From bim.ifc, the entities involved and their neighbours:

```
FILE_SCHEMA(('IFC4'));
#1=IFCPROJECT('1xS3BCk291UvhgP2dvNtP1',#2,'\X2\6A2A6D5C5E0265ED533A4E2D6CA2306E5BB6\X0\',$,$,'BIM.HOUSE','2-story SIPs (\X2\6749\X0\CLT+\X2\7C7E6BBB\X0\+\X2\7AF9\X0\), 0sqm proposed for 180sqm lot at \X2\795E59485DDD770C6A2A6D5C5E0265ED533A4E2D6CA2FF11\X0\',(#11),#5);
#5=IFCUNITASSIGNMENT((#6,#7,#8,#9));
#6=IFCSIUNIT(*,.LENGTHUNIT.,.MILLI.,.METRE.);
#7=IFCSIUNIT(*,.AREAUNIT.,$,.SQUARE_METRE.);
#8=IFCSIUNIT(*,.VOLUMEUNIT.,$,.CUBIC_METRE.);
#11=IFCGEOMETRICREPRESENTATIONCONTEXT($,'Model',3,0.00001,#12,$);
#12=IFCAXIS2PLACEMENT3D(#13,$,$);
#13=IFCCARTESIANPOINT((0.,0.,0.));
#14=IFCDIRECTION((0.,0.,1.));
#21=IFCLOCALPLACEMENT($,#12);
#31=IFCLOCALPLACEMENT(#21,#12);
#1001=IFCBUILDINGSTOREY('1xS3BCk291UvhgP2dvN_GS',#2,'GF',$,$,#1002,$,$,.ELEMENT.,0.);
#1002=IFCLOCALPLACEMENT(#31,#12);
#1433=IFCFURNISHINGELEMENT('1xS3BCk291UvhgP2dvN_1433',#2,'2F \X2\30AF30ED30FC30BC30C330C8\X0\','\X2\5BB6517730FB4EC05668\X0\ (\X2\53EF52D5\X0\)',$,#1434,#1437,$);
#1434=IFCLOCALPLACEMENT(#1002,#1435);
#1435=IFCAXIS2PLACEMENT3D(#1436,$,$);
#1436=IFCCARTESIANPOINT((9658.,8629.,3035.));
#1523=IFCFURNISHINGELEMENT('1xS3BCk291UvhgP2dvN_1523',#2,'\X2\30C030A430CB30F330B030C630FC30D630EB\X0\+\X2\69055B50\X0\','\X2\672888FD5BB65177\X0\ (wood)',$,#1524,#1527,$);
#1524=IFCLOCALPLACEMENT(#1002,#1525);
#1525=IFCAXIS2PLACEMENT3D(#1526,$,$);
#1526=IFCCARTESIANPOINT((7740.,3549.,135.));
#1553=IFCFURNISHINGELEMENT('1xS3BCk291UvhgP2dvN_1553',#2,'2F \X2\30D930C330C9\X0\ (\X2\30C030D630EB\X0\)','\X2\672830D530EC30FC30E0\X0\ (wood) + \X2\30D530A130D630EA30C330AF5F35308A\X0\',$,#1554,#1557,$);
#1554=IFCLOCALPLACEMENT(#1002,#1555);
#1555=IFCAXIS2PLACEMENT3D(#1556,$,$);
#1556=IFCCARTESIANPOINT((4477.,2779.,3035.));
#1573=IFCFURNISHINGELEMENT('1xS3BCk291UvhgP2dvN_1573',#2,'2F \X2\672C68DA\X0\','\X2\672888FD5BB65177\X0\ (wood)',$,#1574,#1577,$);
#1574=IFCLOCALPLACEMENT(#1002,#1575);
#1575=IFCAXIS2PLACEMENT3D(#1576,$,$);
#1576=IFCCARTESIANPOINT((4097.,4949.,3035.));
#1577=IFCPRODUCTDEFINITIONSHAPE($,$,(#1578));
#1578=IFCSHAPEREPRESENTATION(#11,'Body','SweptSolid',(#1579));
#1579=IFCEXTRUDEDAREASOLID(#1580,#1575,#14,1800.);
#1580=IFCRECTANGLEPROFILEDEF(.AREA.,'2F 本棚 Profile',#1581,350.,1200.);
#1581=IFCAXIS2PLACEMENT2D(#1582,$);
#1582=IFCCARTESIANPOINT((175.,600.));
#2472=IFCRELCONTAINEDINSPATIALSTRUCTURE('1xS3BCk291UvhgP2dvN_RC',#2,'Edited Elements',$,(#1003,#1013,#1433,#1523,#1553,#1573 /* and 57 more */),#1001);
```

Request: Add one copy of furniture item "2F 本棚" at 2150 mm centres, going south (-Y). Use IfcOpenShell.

```python
import numpy as np
import ifcopenshell
import ifcopenshell.api.geometry
import ifcopenshell.api.root
import ifcopenshell.util.element
import ifcopenshell.util.placement
import ifcopenshell.util.unit

model = ifcopenshell.open("bim.ifc")
unit_scale = ifcopenshell.util.unit.calculate_unit_scale(model)


def reuse_history(source, copy):
    """copy_class also copies each property set's owner history, people and application; keep the originals."""
    for rel in copy.IsDefinedBy:
        if rel.is_a("IfcRelDefinesByProperties") and (history := rel.RelatingPropertyDefinition.OwnerHistory):
            rel.RelatingPropertyDefinition.OwnerHistory = source.OwnerHistory
            ifcopenshell.util.element.remove_deep2(model, history)


source = model.by_guid("1xS3BCk291UvhgP2dvN_1573")
base = ifcopenshell.util.placement.get_local_placement(source.ObjectPlacement)
step = np.array([0.0, -1.0, 0.0]) * 2.15 / unit_scale

for i in range(1, 2):
    copy = ifcopenshell.api.root.copy_class(model, product=source)
    copy.Representation = ifcopenshell.util.element.copy_deep(
        model, source.Representation, exclude=["IfcGeometricRepresentationContext", "IfcRepresentationMap"]
    )
    reuse_history(source, copy)
    matrix = base.copy()
    matrix[:3, 3] += i * step
    print("added at", matrix[:3, 3].round(3) + 0.0)
    ifcopenshell.api.geometry.edit_object_placement(model, product=copy, matrix=matrix, is_si=False)

model.write("bim_edited.ifc")
```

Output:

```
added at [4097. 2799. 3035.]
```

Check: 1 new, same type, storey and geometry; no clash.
